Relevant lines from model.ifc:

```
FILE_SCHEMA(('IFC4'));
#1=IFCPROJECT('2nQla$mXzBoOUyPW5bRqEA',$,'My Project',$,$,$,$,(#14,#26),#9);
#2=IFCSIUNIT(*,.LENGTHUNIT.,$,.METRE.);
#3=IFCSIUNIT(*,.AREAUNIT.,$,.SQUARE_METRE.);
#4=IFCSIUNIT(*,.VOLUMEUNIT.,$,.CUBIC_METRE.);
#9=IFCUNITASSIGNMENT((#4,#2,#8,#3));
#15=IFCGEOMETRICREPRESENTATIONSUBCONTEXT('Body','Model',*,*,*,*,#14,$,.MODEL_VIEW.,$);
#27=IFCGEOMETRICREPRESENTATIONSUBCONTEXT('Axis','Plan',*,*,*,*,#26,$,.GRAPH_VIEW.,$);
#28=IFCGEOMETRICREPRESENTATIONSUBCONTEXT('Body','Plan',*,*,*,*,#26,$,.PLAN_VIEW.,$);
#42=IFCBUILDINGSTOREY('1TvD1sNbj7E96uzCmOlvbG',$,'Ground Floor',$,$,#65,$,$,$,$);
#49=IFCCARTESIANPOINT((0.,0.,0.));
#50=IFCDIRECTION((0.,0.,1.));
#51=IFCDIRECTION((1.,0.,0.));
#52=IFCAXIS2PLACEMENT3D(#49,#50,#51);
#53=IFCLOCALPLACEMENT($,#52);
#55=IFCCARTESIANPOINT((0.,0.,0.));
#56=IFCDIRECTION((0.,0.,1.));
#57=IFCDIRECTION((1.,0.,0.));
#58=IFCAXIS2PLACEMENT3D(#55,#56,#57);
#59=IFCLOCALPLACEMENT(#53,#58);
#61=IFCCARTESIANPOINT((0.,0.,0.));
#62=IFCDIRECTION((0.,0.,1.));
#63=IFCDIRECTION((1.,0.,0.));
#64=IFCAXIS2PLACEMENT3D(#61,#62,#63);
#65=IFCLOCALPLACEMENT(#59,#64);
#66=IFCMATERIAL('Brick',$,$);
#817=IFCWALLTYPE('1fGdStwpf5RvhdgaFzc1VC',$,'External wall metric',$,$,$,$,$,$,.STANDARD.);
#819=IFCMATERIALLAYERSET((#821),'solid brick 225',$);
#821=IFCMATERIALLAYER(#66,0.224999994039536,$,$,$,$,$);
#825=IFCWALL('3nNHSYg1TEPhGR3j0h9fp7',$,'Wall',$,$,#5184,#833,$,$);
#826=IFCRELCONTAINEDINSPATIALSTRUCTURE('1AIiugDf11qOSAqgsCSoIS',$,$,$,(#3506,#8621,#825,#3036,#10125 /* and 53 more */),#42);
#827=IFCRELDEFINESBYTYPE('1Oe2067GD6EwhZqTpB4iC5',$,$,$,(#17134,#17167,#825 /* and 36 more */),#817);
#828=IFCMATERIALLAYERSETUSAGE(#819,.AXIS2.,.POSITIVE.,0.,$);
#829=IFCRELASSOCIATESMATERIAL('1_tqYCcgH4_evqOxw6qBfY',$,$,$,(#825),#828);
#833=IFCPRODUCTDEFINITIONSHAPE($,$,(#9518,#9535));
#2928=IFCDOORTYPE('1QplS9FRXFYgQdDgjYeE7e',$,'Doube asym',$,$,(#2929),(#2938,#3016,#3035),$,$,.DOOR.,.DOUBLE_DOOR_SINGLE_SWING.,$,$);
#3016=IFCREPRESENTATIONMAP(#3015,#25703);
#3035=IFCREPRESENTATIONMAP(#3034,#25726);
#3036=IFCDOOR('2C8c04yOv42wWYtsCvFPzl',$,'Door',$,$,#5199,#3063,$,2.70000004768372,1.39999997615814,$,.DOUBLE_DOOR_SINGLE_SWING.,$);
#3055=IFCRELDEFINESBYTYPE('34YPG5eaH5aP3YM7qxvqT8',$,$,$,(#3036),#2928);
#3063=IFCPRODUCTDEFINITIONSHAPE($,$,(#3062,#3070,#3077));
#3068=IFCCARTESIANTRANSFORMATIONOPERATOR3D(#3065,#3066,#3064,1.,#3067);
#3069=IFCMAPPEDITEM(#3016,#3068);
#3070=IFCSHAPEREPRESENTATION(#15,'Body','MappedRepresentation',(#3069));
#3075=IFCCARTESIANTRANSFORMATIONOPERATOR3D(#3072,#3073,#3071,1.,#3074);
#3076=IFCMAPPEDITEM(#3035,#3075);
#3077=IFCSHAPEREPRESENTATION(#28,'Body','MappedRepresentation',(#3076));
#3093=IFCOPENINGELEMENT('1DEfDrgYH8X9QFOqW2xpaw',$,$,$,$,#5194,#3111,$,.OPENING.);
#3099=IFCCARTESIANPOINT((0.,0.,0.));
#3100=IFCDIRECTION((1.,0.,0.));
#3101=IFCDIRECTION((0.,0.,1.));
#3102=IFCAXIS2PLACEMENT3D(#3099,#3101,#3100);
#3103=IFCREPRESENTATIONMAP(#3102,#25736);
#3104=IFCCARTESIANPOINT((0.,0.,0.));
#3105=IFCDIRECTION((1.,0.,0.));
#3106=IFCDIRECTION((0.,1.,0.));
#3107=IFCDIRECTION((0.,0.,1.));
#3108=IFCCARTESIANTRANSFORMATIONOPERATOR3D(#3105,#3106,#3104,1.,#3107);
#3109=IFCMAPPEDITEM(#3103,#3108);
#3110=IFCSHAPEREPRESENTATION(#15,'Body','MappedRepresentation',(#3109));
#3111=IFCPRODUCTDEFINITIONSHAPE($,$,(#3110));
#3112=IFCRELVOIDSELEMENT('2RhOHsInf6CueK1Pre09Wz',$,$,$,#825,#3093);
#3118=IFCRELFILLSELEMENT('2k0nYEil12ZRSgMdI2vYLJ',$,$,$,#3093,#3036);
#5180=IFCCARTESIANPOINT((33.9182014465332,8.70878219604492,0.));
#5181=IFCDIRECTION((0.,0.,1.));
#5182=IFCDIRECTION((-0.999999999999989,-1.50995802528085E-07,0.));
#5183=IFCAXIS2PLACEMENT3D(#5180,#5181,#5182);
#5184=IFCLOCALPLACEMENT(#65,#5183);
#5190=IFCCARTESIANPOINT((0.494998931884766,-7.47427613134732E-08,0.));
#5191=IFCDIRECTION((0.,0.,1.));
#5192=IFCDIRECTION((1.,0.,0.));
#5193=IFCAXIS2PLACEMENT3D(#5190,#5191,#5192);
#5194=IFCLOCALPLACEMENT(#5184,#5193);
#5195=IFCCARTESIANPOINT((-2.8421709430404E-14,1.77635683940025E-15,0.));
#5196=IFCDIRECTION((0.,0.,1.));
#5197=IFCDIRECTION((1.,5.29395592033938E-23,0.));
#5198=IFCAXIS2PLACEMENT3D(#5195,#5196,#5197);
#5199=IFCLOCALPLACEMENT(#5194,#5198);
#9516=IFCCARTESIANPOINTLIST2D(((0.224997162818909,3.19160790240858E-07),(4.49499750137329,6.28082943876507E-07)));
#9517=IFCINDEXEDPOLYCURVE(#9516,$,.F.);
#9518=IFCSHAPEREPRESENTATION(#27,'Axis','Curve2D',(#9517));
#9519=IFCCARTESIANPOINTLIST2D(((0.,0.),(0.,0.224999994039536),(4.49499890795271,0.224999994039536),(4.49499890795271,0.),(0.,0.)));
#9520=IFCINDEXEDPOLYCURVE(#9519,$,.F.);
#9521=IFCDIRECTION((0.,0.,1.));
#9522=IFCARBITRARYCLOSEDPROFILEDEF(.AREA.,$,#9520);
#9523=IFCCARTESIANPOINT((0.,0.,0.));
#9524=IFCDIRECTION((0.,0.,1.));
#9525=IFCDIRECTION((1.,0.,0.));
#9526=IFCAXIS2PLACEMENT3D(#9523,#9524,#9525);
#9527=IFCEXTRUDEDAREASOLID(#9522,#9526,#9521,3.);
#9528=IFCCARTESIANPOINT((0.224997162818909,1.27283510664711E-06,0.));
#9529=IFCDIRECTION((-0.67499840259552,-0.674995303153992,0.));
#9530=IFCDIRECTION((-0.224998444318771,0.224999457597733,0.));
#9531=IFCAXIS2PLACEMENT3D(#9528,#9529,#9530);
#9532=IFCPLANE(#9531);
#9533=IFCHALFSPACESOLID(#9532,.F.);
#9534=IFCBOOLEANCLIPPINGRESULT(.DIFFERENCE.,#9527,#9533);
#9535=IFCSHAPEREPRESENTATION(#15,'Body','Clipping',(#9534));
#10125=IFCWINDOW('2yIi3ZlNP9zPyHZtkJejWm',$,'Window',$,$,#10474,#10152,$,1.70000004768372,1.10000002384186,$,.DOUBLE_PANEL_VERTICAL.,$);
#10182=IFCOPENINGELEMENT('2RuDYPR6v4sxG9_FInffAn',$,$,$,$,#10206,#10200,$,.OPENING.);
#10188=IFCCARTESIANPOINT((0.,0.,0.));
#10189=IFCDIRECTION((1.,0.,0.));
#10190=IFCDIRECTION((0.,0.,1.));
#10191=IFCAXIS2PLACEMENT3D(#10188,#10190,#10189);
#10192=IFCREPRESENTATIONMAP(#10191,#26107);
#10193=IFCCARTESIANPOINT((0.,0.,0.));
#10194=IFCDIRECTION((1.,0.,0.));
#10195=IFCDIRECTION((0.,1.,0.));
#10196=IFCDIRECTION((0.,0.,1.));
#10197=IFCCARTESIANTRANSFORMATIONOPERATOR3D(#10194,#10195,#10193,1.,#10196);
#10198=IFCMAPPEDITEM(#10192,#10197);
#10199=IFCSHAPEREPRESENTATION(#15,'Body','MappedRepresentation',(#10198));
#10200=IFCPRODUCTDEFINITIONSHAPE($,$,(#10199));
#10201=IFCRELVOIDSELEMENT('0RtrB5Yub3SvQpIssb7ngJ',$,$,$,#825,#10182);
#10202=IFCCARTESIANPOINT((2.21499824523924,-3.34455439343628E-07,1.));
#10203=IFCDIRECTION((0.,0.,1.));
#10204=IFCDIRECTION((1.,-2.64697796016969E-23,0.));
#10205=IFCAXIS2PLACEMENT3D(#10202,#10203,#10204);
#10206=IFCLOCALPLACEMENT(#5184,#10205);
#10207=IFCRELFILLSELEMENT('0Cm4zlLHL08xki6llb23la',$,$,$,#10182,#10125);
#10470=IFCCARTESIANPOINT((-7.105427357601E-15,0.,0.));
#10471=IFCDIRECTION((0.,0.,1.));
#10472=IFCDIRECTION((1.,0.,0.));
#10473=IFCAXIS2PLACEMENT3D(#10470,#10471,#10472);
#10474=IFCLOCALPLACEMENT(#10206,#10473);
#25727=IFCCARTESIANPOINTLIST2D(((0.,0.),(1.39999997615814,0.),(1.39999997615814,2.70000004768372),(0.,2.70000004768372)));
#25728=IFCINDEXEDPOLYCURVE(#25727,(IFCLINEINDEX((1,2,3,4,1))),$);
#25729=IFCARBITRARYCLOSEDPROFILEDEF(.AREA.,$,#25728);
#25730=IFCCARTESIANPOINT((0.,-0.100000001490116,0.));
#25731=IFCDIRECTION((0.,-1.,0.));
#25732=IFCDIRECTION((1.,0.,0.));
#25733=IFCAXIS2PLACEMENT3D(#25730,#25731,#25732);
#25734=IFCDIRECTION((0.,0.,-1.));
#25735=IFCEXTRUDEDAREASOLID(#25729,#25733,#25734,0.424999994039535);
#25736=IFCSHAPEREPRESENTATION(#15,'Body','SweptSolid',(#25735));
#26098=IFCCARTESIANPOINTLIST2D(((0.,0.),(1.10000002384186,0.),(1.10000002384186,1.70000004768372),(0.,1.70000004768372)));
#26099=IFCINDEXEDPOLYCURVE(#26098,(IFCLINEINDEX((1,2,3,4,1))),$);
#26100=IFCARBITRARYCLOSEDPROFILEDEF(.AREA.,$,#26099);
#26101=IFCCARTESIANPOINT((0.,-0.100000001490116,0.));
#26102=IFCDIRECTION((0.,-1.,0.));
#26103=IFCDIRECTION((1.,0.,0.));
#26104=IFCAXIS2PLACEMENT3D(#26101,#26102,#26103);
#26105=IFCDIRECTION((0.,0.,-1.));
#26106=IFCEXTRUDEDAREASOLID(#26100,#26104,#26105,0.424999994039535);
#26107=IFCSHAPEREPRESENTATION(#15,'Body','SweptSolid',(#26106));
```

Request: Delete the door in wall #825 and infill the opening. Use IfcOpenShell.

```python
import ifcopenshell
import ifcopenshell.api.feature
import ifcopenshell.api.root
import ifcopenshell.geom
import ifcopenshell.util.shape

model = ifcopenshell.open("model.ifc")
settings = ifcopenshell.geom.settings()


def volume(element):
    """Net volume in cubic metres, openings subtracted."""
    shape = ifcopenshell.geom.create_shape(settings, element)
    return ifcopenshell.util.shape.get_volume(shape.geometry)


door = model.by_id(3036)
opening = door.FillsVoids[0].RelatingOpeningElement
wall = opening.VoidsElements[0].RelatingBuildingElement
before = volume(wall)

ifcopenshell.api.root.remove_product(model, product=door)
ifcopenshell.api.feature.remove_feature(model, feature=opening)

after = volume(wall)

print(f"wall volume {before:.3f} -> {after:.3f} m3")

model.write("model_v2.ifc")
```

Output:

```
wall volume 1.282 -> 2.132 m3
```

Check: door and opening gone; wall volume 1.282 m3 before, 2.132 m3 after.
